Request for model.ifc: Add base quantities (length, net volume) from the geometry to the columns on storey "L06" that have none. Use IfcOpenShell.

First a look at what the model holds.

```python
import ifcopenshell
import ifcopenshell.util.element
import ifcopenshell.util.unit

model = ifcopenshell.open("model.ifc")
print(model.schema)
for unit_type in ("LENGTHUNIT", "AREAUNIT", "VOLUMEUNIT"):
    print(unit_type, ifcopenshell.util.unit.calculate_unit_scale(model, unit_type))
storey = next(s for s in model.by_type("IfcBuildingStorey") if s.Name == "L06")
columns = [e for e in ifcopenshell.util.element.get_decomposition(storey) if e.is_a("IfcColumn")]
for e in sorted(columns, key=lambda e: e.id()):
    print(e.id(), e.is_a(), e.Name, list(ifcopenshell.util.element.get_psets(e, qtos_only=True)), sep=" | ")
```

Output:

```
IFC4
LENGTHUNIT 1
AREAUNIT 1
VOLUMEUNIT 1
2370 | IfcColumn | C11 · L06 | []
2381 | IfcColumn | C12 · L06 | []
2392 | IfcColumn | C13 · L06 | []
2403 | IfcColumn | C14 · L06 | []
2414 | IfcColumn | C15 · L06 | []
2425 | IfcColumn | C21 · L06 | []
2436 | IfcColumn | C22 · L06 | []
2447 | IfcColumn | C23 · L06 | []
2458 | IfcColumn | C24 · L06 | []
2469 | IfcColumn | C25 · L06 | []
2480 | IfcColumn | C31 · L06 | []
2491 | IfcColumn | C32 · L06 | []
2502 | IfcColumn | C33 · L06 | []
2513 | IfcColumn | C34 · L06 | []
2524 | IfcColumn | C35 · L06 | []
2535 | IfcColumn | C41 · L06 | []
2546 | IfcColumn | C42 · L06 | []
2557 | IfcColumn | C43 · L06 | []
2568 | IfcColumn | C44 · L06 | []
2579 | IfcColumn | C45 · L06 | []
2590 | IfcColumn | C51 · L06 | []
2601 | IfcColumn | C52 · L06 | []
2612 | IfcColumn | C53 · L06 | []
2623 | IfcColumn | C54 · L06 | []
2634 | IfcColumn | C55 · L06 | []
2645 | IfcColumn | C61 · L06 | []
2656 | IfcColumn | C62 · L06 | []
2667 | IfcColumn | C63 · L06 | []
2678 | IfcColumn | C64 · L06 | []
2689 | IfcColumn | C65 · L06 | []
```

```python
import ifcopenshell
import ifcopenshell.api.pset
import ifcopenshell.geom
import ifcopenshell.util.element
import ifcopenshell.util.shape
import ifcopenshell.util.unit

model = ifcopenshell.open("model.ifc")
unit_scale = ifcopenshell.util.unit.calculate_unit_scale(model)
volume_scale = ifcopenshell.util.unit.calculate_unit_scale(model, "VOLUMEUNIT")
settings = ifcopenshell.geom.settings()

storey = next(s for s in model.by_type("IfcBuildingStorey") if s.Name == "L06")
columns = [e for e in ifcopenshell.util.element.get_decomposition(storey) if e.is_a("IfcColumn")]

for e in sorted(columns, key=lambda e: e.id()):
    if ifcopenshell.util.element.get_psets(e, qtos_only=True, should_inherit=False):
        continue
    # Geometry comes back in metres, in the element's own axes.
    shape = ifcopenshell.geom.create_shape(settings, e)
    values = {
        "Length": ifcopenshell.util.shape.get_z(shape.geometry) / unit_scale,
        "NetVolume": ifcopenshell.util.shape.get_volume(shape.geometry) / volume_scale,
    }
    qto = ifcopenshell.api.pset.add_qto(model, product=e, name="Qto_ColumnBaseQuantities")
    ifcopenshell.api.pset.edit_qto(model, qto=qto, properties=values)
    print(e.id(), {k: round(v, 3) for k, v in values.items()})

model.write("model_updated.ifc")
```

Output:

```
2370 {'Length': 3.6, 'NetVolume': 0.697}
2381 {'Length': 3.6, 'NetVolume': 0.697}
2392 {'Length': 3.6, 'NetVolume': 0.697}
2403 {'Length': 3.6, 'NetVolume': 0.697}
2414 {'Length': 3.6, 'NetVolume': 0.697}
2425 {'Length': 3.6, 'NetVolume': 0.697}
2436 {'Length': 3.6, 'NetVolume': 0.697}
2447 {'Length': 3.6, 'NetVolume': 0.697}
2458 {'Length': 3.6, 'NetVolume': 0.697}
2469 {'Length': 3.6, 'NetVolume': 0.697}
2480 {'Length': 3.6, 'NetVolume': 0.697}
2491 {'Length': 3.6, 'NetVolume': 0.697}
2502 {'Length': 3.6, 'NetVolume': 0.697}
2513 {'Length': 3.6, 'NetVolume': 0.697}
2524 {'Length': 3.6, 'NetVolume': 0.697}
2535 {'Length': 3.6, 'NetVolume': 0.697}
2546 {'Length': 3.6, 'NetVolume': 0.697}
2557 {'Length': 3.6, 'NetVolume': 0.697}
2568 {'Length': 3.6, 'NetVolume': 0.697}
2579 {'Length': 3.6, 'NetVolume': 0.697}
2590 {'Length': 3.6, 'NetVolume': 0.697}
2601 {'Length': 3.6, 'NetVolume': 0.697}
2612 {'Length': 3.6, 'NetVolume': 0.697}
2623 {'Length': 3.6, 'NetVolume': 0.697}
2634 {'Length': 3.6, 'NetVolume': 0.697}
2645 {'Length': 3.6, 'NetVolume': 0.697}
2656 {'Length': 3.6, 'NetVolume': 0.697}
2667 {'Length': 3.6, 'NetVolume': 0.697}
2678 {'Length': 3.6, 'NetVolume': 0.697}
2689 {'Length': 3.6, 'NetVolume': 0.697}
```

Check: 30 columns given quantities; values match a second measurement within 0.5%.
